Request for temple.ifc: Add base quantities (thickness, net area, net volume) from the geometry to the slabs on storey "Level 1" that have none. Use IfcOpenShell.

First a look at what the model holds.

```python
import ifcopenshell
import ifcopenshell.util.element
import ifcopenshell.util.unit

model = ifcopenshell.open("temple.ifc")
print(model.schema)
for unit_type in ("LENGTHUNIT", "AREAUNIT", "VOLUMEUNIT"):
    print(unit_type, ifcopenshell.util.unit.calculate_unit_scale(model, unit_type))
storey = next(s for s in model.by_type("IfcBuildingStorey") if s.Name == "Level 1")
slabs = [e for e in ifcopenshell.util.element.get_decomposition(storey) if e.is_a("IfcSlab")]
for e in sorted(slabs, key=lambda e: e.id()):
    print(e.id(), e.is_a(), e.Name, list(ifcopenshell.util.element.get_psets(e, qtos_only=True)), sep=" | ")
```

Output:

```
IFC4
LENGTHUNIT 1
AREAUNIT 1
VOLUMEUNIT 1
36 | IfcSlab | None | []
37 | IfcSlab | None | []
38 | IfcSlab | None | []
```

```python
import ifcopenshell
import ifcopenshell.api.pset
import ifcopenshell.geom
import ifcopenshell.util.element
import ifcopenshell.util.shape
import ifcopenshell.util.unit

model = ifcopenshell.open("temple.ifc")
unit_scale = ifcopenshell.util.unit.calculate_unit_scale(model)
area_scale = ifcopenshell.util.unit.calculate_unit_scale(model, "AREAUNIT")
volume_scale = ifcopenshell.util.unit.calculate_unit_scale(model, "VOLUMEUNIT")
settings = ifcopenshell.geom.settings()

storey = next(s for s in model.by_type("IfcBuildingStorey") if s.Name == "Level 1")
slabs = [e for e in ifcopenshell.util.element.get_decomposition(storey) if e.is_a("IfcSlab")]

for e in sorted(slabs, key=lambda e: e.id()):
    if ifcopenshell.util.element.get_psets(e, qtos_only=True, should_inherit=False):
        continue
    # Geometry comes back in metres, in the element's own axes.
    shape = ifcopenshell.geom.create_shape(settings, e)
    values = {
        "Width": ifcopenshell.util.shape.get_z(shape.geometry) / unit_scale,
        "NetArea": ifcopenshell.util.shape.get_footprint_area(shape.geometry) / area_scale,
        "NetVolume": ifcopenshell.util.shape.get_volume(shape.geometry) / volume_scale,
    }
    qto = ifcopenshell.api.pset.add_qto(model, product=e, name="Qto_SlabBaseQuantities")
    ifcopenshell.api.pset.edit_qto(model, qto=qto, properties=values)
    print(e.id(), {k: round(v, 3) for k, v in values.items()})

model.write("temple_updated.ifc")
```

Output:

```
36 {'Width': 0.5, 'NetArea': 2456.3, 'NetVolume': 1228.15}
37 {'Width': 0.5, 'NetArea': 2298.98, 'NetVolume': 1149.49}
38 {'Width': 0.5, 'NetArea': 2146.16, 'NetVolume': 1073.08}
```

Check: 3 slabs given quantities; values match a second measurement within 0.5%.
